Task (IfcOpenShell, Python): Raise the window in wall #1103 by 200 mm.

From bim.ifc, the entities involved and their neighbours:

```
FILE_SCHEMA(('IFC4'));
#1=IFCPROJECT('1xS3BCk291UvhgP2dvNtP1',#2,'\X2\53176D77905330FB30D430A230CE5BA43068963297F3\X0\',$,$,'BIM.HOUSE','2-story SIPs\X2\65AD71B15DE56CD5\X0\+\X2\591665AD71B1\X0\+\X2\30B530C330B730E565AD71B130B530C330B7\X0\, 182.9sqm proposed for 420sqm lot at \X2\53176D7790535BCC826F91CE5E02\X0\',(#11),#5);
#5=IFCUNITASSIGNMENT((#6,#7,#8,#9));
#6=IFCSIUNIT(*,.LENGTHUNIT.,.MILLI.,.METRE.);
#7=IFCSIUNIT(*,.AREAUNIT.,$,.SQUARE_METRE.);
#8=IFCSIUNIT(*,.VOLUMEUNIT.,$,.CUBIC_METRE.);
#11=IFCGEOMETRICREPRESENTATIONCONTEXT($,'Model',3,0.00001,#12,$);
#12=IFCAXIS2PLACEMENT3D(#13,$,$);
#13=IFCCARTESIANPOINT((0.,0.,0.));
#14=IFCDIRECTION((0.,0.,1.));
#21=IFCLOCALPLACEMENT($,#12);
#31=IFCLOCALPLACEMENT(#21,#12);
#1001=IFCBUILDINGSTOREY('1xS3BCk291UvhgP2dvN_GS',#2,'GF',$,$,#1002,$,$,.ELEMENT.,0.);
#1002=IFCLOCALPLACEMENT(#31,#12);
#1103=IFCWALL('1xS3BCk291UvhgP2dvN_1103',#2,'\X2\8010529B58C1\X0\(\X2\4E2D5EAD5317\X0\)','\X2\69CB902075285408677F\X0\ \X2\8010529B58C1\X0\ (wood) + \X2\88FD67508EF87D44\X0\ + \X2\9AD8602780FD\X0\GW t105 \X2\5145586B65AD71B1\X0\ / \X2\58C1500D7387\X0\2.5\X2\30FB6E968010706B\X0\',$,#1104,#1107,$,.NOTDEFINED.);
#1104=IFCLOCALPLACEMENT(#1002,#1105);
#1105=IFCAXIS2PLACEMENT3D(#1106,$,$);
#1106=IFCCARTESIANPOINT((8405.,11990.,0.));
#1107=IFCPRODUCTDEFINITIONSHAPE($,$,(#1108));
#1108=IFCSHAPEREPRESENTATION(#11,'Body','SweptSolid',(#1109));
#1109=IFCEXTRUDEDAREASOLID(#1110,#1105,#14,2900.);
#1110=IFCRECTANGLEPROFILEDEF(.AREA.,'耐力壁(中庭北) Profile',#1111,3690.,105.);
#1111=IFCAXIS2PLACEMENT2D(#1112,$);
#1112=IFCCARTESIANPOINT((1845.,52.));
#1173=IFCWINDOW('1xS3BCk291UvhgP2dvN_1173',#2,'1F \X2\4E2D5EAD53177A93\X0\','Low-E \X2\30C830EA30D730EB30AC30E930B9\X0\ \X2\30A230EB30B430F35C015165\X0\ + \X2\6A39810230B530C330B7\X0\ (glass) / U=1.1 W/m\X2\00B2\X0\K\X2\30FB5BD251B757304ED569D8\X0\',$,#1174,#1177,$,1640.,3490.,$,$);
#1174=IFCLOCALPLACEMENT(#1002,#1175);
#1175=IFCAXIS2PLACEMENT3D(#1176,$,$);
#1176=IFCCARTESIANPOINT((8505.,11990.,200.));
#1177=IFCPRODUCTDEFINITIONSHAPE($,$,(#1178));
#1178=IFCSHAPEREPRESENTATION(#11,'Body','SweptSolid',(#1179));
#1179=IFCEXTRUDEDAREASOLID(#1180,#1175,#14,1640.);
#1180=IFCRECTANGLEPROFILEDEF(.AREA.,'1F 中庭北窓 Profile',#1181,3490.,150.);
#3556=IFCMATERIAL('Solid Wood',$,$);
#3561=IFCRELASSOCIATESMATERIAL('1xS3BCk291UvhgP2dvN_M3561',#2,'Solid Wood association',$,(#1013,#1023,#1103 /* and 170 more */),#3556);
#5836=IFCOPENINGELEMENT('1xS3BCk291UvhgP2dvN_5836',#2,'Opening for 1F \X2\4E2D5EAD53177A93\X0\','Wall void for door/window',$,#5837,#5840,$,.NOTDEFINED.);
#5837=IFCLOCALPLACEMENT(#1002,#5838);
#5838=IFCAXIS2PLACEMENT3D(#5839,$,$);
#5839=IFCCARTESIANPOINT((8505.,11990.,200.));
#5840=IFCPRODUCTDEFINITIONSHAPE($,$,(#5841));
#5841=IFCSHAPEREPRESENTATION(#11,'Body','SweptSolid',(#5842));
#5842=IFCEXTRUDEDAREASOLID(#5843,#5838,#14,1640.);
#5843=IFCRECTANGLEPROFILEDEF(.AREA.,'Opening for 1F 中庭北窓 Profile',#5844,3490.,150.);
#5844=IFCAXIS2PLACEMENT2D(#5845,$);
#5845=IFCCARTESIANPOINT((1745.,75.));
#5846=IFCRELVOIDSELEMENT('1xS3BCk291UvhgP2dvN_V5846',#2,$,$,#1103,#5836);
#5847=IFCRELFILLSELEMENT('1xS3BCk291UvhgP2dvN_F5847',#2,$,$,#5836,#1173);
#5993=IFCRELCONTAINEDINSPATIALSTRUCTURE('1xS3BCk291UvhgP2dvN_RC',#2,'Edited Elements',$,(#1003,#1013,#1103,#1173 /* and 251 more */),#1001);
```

```python
import numpy as np
import ifcopenshell
import ifcopenshell.api.geometry
import ifcopenshell.util.placement
import ifcopenshell.util.unit

model = ifcopenshell.open("bim.ifc")
unit_scale = ifcopenshell.util.unit.calculate_unit_scale(model)

window = model.by_guid("1xS3BCk291UvhgP2dvN_1173")
opening = window.FillsVoids[0].RelatingOpeningElement
dz = 200.0

shift = np.array([0.0, 0.0, dz])
# The window is not placed relative to its opening, so move both.
for product in (opening, window):
    matrix = ifcopenshell.util.placement.get_local_placement(product.ObjectPlacement)
    matrix[:3, 3] += shift
    ifcopenshell.api.geometry.edit_object_placement(model, product=product, matrix=matrix, is_si=False)

print(f"moved by {dz * unit_scale:+.3f} m")

model.write("bim-out.ifc")
```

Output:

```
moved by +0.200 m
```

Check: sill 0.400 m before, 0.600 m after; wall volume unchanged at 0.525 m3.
